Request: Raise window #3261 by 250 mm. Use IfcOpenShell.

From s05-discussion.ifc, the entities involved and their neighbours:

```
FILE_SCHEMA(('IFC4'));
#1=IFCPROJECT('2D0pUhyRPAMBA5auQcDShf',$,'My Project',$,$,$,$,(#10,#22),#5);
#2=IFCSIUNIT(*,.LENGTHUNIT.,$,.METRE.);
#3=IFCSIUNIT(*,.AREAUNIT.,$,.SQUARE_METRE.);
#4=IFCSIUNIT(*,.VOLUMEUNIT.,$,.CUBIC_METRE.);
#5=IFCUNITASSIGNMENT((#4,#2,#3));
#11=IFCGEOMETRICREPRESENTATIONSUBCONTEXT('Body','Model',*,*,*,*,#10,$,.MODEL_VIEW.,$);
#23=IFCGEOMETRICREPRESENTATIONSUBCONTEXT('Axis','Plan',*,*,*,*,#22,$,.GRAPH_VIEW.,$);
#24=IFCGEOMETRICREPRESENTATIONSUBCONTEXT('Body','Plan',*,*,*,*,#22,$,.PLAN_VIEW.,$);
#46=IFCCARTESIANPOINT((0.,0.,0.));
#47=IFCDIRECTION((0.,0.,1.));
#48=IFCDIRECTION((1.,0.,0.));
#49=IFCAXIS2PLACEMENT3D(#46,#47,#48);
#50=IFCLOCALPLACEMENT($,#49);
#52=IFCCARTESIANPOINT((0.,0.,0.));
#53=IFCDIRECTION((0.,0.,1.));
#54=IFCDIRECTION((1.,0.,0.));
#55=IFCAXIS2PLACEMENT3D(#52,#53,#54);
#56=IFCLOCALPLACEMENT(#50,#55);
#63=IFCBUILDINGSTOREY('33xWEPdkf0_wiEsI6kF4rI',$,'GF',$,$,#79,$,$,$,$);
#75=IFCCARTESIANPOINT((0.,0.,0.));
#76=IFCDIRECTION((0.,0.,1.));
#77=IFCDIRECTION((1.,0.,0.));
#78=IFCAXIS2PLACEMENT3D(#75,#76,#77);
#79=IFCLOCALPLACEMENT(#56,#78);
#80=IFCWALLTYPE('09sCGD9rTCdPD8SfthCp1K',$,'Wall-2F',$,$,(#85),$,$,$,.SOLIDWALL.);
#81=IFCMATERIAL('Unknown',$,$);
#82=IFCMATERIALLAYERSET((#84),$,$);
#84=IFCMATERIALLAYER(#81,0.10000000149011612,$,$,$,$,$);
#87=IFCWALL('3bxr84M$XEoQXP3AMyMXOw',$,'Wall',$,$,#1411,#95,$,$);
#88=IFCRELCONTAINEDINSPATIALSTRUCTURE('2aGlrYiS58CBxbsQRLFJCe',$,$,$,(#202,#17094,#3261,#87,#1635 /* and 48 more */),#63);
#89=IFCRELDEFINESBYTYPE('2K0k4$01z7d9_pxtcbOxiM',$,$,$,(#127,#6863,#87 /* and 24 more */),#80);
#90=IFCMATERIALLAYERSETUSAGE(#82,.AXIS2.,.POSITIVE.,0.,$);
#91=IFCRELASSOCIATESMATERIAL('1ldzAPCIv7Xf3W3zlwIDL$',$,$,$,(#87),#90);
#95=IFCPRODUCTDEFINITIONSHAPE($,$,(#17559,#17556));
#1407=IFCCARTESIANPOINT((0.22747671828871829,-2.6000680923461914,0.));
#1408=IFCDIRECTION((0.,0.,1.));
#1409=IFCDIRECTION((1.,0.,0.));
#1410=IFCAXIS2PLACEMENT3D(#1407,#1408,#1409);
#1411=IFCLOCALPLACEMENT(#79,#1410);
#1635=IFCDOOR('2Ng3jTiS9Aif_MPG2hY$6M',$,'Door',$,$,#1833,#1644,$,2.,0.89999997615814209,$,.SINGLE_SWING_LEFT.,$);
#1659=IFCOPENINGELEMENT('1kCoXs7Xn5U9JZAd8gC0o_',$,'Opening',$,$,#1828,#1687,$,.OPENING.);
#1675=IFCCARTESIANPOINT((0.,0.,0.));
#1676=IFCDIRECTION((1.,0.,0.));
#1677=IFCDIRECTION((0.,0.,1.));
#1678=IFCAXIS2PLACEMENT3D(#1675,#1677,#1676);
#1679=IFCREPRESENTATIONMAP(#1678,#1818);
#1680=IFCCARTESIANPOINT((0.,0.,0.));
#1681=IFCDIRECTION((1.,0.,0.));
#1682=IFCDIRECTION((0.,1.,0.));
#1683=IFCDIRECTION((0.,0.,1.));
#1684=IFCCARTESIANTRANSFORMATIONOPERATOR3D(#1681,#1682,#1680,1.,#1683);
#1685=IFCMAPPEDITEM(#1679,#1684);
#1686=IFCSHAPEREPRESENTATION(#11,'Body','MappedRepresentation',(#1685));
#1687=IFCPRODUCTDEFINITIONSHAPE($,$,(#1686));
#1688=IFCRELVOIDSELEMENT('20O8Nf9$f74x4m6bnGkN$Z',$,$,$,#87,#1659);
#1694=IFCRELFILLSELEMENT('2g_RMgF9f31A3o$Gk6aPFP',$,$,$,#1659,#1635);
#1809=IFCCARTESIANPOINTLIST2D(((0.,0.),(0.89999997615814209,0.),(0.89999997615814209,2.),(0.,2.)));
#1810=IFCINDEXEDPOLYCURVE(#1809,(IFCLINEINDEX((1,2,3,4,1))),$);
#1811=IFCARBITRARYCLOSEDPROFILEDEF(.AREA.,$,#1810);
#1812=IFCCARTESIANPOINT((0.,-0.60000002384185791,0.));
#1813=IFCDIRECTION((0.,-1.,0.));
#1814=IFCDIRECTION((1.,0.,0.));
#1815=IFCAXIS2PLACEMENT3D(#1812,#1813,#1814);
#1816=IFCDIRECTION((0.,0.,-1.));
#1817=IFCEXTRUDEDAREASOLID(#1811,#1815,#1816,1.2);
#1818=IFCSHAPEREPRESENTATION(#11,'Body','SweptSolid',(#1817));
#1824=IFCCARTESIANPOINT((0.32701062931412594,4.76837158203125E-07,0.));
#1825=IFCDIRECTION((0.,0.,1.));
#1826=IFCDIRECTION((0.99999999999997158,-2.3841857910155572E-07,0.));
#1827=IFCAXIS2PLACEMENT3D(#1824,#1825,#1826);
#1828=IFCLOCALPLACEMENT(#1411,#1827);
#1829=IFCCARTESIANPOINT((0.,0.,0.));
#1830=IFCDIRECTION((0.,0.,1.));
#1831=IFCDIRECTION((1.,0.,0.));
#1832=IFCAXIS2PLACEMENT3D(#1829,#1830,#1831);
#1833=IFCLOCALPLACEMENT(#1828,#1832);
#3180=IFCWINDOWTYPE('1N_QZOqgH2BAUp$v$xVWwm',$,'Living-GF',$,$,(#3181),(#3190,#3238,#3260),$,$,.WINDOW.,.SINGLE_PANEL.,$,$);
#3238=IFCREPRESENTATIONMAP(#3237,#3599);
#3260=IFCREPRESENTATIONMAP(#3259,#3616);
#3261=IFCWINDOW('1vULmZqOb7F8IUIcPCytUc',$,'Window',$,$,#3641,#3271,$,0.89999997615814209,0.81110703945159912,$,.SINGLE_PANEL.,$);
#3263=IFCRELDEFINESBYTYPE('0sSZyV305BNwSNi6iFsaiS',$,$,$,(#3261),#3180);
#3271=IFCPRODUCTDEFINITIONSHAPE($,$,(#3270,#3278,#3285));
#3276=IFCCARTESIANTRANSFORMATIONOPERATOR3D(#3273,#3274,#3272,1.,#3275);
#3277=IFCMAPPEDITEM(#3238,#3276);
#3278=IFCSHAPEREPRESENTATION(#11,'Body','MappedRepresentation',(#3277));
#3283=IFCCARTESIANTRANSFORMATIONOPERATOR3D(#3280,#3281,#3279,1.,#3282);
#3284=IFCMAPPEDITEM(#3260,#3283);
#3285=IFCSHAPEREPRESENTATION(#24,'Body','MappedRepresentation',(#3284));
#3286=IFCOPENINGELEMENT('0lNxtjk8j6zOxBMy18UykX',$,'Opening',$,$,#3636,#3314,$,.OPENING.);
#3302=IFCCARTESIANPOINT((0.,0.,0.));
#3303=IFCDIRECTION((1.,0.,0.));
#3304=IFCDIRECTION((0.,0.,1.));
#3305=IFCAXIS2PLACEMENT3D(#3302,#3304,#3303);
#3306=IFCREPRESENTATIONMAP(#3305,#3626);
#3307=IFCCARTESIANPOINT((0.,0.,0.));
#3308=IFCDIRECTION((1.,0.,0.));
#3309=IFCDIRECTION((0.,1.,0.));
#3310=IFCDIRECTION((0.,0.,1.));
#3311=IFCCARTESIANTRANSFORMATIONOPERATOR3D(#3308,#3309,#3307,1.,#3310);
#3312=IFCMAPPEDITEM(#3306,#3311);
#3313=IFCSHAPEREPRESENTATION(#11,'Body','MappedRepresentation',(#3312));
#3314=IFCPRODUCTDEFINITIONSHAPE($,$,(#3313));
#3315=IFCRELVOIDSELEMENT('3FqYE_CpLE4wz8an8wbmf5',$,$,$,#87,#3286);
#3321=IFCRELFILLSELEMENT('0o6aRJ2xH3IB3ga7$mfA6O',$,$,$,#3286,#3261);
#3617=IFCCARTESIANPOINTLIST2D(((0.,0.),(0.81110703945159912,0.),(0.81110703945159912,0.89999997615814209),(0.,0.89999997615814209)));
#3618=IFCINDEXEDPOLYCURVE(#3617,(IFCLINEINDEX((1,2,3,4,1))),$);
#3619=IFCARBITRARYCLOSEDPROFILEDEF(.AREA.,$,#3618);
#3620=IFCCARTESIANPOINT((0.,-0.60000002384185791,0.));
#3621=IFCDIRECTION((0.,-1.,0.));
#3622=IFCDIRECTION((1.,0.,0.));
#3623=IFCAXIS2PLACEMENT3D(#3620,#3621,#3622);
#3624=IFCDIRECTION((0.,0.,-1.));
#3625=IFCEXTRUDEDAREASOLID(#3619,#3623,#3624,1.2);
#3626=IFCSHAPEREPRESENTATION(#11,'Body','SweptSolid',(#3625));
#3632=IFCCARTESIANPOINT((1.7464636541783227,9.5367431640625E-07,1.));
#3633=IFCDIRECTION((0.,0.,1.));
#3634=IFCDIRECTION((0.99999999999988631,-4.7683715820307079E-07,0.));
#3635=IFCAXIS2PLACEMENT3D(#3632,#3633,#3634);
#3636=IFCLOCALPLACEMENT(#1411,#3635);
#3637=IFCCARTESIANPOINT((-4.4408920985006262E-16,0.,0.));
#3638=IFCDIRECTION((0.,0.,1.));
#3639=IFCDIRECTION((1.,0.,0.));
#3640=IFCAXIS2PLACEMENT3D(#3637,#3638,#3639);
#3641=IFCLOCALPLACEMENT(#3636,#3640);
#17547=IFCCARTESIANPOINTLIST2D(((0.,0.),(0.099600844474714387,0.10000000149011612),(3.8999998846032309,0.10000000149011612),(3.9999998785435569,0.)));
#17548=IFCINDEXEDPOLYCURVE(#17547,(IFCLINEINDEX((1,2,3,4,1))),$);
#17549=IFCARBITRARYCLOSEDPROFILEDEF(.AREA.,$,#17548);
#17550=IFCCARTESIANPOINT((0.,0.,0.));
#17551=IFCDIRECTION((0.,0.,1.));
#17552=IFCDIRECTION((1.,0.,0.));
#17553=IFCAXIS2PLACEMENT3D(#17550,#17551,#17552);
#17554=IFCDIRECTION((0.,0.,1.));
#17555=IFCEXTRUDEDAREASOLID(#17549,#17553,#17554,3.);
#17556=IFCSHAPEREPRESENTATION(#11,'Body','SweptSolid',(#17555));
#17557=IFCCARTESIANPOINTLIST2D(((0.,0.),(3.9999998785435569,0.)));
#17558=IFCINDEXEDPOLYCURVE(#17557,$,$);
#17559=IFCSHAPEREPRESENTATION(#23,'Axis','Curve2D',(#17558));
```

```python
import numpy as np
import ifcopenshell
import ifcopenshell.api.geometry
import ifcopenshell.util.placement
import ifcopenshell.util.unit

model = ifcopenshell.open("s05-discussion.ifc")
unit_scale = ifcopenshell.util.unit.calculate_unit_scale(model)

window = model.by_guid("1vULmZqOb7F8IUIcPCytUc")
opening = window.FillsVoids[0].RelatingOpeningElement
dz = 0.25 / unit_scale

shift = np.array([0.0, 0.0, dz])
# The window is placed relative to its opening, so it follows when the opening moves.
matrix = ifcopenshell.util.placement.get_local_placement(opening.ObjectPlacement)
matrix[:3, 3] += shift
ifcopenshell.api.geometry.edit_object_placement(
    model, product=opening, matrix=matrix, is_si=False, should_transform_children=True
)

print(f"moved by {dz * unit_scale:+.3f} m")

model.write("s05-discussion_v2.ifc")
```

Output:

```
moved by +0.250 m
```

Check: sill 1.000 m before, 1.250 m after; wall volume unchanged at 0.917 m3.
